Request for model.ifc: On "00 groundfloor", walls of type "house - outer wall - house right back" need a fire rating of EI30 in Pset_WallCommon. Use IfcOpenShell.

First a look at what the model holds.

```python
import ifcopenshell
import ifcopenshell.util.element

model = ifcopenshell.open("model.ifc")
print(model.schema)
storey = next(s for s in model.by_type("IfcBuildingStorey") if s.Name == "00 groundfloor")
walls = [e for e in ifcopenshell.util.element.get_decomposition(storey) if e.is_a("IfcWall")]
seen = {}
for e in walls:
    element_type = ifcopenshell.util.element.get_type(e)
    key = (element_type.Name if element_type != e and element_type else None, ifcopenshell.util.element.get_pset(e, "Pset_WallCommon", "FireRating"))
    seen[key] = seen.get(key, 0) + 1
for (name, value), count in sorted(seen.items(), key=str):
    print(count, "x", name, "|", value)
```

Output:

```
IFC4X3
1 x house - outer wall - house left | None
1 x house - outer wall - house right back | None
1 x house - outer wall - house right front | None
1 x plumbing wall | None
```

```python
import ifcopenshell
import ifcopenshell.api.pset
import ifcopenshell.util.element

model = ifcopenshell.open("model.ifc")

storey = next(s for s in model.by_type("IfcBuildingStorey") if s.Name == "00 groundfloor")
walls = [e for e in ifcopenshell.util.element.get_decomposition(storey) if e.is_a("IfcWall")]

count = 0
for e in walls:
    element_type = ifcopenshell.util.element.get_type(e)
    if element_type in (None, e) or element_type.Name != "house - outer wall - house right back":
        continue
    # add_pset returns the element's existing set when there is one.
    pset = ifcopenshell.api.pset.add_pset(model, product=e, name="Pset_WallCommon")
    ifcopenshell.api.pset.edit_pset(model, pset=pset, properties={"FireRating": "EI30"})
    count += 1

print(count, "walls updated")

model.write("model_updated.ifc")
```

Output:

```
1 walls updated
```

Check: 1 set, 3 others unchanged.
